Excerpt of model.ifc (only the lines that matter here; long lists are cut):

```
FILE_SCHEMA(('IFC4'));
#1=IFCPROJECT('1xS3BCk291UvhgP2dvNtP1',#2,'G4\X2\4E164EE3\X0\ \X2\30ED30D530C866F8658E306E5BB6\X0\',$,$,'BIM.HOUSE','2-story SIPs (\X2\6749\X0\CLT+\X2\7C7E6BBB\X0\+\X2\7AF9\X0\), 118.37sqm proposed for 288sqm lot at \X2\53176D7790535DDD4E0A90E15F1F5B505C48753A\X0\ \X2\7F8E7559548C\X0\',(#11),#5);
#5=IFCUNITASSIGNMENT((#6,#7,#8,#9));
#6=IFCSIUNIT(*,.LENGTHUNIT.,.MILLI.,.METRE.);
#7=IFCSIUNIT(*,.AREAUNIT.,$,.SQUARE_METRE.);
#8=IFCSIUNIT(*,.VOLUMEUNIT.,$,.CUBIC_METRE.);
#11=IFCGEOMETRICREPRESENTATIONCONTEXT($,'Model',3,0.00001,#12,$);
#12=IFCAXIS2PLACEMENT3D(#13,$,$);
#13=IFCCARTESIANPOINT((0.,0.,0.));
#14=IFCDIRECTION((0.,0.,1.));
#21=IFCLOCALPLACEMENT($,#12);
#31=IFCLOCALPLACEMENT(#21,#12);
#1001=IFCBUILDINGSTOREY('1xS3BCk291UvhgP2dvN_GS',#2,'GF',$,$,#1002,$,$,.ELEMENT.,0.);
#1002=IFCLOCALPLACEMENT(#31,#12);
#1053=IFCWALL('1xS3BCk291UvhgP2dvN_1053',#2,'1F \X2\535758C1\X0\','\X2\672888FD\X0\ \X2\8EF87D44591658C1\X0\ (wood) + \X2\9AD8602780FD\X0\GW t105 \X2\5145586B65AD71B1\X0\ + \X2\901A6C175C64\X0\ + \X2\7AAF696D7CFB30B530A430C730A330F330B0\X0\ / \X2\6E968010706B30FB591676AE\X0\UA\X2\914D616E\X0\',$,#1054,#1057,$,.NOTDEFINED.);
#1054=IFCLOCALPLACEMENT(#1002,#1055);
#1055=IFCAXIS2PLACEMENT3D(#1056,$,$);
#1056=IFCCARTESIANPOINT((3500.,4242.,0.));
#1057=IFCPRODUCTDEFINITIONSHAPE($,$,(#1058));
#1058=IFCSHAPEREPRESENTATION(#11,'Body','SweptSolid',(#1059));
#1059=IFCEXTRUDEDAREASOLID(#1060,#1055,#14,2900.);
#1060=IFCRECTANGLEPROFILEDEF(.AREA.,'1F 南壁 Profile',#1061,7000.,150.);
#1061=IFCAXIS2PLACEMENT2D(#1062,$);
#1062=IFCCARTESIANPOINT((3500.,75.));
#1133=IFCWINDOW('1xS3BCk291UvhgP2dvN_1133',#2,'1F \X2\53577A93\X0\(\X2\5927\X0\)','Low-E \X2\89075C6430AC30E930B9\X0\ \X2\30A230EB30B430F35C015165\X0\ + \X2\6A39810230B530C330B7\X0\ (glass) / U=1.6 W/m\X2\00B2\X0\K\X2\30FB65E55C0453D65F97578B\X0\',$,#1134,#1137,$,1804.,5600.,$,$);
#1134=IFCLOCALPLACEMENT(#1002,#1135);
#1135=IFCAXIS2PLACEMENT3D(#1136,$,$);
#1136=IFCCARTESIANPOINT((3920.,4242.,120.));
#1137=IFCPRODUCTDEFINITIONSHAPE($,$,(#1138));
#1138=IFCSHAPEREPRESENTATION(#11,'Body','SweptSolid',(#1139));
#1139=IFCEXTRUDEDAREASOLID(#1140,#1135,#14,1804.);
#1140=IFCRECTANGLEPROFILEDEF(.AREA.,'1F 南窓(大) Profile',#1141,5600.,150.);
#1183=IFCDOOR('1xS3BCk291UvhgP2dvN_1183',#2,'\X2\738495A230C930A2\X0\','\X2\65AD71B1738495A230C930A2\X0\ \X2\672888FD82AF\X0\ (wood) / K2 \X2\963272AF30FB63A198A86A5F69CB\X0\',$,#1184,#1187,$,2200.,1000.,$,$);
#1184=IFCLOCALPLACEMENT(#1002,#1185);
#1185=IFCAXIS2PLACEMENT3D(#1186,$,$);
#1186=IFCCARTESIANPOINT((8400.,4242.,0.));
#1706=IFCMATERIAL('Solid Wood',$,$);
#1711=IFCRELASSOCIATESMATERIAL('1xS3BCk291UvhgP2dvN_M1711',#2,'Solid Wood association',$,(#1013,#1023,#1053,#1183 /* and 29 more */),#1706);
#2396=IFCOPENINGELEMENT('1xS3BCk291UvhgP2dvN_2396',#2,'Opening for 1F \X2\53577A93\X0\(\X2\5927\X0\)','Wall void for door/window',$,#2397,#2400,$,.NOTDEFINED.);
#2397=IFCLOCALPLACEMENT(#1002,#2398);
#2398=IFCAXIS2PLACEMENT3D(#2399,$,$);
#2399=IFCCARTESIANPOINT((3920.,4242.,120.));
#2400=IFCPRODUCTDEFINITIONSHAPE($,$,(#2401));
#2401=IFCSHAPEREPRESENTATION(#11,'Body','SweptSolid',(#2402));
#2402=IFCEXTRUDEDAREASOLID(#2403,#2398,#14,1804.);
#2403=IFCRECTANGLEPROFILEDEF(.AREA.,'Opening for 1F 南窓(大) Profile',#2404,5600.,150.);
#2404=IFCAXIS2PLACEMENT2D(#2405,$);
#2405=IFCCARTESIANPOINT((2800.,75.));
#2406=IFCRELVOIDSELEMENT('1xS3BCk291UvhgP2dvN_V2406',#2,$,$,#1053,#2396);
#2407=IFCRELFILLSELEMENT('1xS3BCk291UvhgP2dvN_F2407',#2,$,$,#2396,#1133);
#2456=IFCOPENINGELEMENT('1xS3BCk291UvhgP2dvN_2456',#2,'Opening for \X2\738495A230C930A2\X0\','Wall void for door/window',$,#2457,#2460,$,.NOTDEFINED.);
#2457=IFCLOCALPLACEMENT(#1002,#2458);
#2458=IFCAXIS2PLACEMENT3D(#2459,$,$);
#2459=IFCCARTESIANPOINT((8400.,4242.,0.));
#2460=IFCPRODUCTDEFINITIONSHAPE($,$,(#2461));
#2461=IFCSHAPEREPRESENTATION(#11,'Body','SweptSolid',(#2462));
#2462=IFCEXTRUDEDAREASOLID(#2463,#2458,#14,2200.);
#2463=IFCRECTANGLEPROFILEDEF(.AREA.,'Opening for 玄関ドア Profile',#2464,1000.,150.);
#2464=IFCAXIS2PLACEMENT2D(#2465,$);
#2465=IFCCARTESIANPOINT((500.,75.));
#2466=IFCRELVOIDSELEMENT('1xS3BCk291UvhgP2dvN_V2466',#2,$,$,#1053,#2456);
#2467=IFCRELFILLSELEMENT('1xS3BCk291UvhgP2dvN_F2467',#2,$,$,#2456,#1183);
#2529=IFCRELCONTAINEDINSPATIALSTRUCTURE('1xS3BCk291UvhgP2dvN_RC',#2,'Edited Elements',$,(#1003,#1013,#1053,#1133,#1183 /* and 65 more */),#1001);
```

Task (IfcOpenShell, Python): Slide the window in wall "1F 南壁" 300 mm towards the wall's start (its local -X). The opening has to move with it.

```python
import ifcopenshell
import ifcopenshell.api.geometry
import ifcopenshell.util.placement

model = ifcopenshell.open("model.ifc")

window = model.by_id(1133)
opening = window.FillsVoids[0].RelatingOpeningElement
wall = opening.VoidsElements[0].RelatingBuildingElement

wall_matrix = ifcopenshell.util.placement.get_local_placement(wall.ObjectPlacement)
shift = wall_matrix[:3, 0] * -300.0
before = ifcopenshell.util.placement.get_local_placement(window.ObjectPlacement)[:3, 3].copy()

# The window is not placed relative to its opening, so move both.
for product in (opening, window):
    matrix = ifcopenshell.util.placement.get_local_placement(product.ObjectPlacement)
    matrix[:3, 3] += shift
    ifcopenshell.api.geometry.edit_object_placement(model, product=product, matrix=matrix, is_si=False)

after = ifcopenshell.util.placement.get_local_placement(window.ObjectPlacement)[:3, 3]
print("window moved by", (after - before).round(3) + 0.0)

model.write("model_v2.ifc")
```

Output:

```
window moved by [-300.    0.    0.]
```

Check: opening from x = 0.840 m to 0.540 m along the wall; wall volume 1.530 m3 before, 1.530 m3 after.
